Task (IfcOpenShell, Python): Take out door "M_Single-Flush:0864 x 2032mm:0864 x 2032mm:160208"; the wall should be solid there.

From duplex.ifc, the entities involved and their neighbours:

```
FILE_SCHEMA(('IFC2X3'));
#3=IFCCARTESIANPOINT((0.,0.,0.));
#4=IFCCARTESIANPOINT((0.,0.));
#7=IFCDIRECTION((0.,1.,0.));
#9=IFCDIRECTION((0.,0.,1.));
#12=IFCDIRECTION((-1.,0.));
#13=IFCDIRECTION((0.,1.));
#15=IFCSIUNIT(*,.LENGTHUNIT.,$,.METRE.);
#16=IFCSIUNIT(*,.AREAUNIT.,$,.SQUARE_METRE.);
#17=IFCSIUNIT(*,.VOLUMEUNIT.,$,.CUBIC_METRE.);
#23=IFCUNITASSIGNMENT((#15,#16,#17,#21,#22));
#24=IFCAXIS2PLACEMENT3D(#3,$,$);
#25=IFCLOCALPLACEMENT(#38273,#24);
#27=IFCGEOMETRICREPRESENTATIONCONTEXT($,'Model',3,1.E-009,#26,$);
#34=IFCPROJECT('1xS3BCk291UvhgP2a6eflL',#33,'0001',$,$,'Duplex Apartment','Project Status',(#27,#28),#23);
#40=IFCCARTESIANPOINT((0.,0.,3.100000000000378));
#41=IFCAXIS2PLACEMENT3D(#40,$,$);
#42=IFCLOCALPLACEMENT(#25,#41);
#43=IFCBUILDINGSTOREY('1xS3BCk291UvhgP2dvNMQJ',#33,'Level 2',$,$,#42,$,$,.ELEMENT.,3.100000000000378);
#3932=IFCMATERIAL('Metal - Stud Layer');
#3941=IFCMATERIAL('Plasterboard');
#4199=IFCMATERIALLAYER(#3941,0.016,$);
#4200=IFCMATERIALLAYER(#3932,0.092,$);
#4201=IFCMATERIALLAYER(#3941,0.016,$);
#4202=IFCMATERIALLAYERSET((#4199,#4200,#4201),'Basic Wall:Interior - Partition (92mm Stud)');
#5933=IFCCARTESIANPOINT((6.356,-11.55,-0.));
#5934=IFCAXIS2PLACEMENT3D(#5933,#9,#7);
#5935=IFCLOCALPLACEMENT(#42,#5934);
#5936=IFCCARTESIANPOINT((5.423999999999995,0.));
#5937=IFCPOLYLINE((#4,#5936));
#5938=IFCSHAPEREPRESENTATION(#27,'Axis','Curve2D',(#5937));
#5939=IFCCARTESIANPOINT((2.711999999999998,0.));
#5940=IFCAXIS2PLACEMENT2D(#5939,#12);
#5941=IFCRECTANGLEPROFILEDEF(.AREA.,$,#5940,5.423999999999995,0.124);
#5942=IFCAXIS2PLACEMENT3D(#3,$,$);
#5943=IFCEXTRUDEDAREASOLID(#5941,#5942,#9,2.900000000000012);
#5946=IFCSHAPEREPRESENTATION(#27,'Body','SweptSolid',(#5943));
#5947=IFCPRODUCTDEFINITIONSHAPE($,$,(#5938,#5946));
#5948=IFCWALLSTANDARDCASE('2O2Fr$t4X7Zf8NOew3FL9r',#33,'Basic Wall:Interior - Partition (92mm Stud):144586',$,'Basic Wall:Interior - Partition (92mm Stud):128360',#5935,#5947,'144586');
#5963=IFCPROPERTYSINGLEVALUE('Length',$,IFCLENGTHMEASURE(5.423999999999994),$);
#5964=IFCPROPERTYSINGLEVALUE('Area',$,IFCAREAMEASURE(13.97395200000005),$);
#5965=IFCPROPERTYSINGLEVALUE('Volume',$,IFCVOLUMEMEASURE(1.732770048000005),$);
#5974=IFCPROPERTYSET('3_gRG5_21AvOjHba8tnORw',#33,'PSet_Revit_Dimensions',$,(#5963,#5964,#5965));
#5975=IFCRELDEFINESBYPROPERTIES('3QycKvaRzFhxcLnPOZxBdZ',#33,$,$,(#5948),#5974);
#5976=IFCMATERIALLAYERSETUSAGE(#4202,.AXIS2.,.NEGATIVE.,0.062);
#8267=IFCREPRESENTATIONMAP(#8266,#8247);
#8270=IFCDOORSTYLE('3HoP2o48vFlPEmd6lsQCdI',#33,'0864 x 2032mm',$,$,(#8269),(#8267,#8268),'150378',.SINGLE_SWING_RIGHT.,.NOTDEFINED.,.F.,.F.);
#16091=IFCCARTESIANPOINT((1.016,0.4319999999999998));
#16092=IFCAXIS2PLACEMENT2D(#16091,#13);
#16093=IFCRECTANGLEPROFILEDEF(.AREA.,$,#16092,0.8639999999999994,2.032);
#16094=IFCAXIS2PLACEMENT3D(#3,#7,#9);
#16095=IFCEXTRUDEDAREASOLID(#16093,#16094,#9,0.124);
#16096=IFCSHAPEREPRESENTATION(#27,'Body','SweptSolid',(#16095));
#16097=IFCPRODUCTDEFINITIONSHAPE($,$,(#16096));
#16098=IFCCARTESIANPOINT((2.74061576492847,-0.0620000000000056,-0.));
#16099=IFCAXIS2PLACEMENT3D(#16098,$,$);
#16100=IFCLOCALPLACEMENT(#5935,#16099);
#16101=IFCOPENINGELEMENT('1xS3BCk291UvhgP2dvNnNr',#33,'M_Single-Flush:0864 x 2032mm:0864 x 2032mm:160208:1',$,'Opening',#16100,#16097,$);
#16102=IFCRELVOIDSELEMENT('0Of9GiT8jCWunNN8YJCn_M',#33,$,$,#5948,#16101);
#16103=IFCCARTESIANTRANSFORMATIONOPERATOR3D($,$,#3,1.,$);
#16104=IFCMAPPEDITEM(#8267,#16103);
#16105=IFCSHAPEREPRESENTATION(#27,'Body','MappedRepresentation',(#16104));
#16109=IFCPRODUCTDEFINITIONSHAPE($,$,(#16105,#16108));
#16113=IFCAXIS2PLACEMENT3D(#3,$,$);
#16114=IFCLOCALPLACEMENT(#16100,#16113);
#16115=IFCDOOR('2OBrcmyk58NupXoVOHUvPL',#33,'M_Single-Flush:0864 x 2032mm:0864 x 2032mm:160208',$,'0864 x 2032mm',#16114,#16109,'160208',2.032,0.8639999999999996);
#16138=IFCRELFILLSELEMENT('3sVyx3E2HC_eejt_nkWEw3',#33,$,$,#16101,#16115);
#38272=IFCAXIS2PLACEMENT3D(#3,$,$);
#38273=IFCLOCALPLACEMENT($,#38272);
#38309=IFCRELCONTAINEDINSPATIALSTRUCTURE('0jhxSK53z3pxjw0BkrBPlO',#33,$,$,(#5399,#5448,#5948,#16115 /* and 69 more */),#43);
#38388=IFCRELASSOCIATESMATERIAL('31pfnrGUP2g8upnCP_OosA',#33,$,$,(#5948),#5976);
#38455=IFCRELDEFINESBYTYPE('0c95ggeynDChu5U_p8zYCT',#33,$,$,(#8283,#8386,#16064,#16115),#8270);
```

```python
import ifcopenshell
import ifcopenshell.api.feature
import ifcopenshell.api.pset
import ifcopenshell.api.root
import ifcopenshell.geom
import ifcopenshell.util.element
import ifcopenshell.util.shape
import ifcopenshell.util.unit

model = ifcopenshell.open("duplex.ifc")
area_scale = ifcopenshell.util.unit.calculate_unit_scale(model, "AREAUNIT")
volume_scale = ifcopenshell.util.unit.calculate_unit_scale(model, "VOLUMEUNIT")
settings = ifcopenshell.geom.settings()


def volume(element):
    """Net volume in cubic metres, openings subtracted."""
    shape = ifcopenshell.geom.create_shape(settings, element)
    return ifcopenshell.util.shape.get_volume(shape.geometry)


door = model.by_guid("2OBrcmyk58NupXoVOHUvPL")
opening = door.FillsVoids[0].RelatingOpeningElement
wall = opening.VoidsElements[0].RelatingBuildingElement
before = volume(wall)

ifcopenshell.api.root.remove_product(model, product=door)
ifcopenshell.api.feature.remove_feature(model, feature=opening)

after = volume(wall)
thickness = 0.124  # wall thickness in metres

# Update the wall's stored quantities.
pset = model.by_id(ifcopenshell.util.element.get_pset(wall, "PSet_Revit_Dimensions", should_inherit=False)["id"])
ifcopenshell.api.pset.edit_pset(model, pset=pset, properties={
    "Area": model.create_entity("IfcAreaMeasure", after / thickness / area_scale),
    "Volume": model.create_entity("IfcVolumeMeasure", after / volume_scale),
})

print(f"wall volume {before:.3f} -> {after:.3f} m3")

model.write("duplex_rev.ifc")
```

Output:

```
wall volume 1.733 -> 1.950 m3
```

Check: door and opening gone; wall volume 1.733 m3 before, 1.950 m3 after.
